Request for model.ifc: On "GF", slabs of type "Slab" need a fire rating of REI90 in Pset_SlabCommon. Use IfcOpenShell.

First a look at what the model holds.

```python
import ifcopenshell
import ifcopenshell.util.element

model = ifcopenshell.open("model.ifc")
print(model.schema)
storey = next(s for s in model.by_type("IfcBuildingStorey") if s.Name == "GF")
slabs = [e for e in ifcopenshell.util.element.get_decomposition(storey) if e.is_a("IfcSlab")]
seen = {}
for e in slabs:
    element_type = ifcopenshell.util.element.get_type(e)
    key = (element_type.Name if element_type != e and element_type else None, ifcopenshell.util.element.get_pset(e, "Pset_SlabCommon", "FireRating"))
    seen[key] = seen.get(key, 0) + 1
for (name, value), count in sorted(seen.items(), key=str):
    print(count, "x", name, "|", value)
```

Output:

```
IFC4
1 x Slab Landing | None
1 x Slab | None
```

```python
import ifcopenshell
import ifcopenshell.api.pset
import ifcopenshell.util.element

model = ifcopenshell.open("model.ifc")

storey = next(s for s in model.by_type("IfcBuildingStorey") if s.Name == "GF")
slabs = [e for e in ifcopenshell.util.element.get_decomposition(storey) if e.is_a("IfcSlab")]

count = 0
for e in slabs:
    element_type = ifcopenshell.util.element.get_type(e)
    if element_type in (None, e) or element_type.Name != "Slab":
        continue
    # add_pset returns the element's existing set when there is one.
    pset = ifcopenshell.api.pset.add_pset(model, product=e, name="Pset_SlabCommon")
    ifcopenshell.api.pset.edit_pset(model, pset=pset, properties={"FireRating": "REI90"})
    count += 1

print(count, "slabs updated")

model.write("model_edited.ifc")
```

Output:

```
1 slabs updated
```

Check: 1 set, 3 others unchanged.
